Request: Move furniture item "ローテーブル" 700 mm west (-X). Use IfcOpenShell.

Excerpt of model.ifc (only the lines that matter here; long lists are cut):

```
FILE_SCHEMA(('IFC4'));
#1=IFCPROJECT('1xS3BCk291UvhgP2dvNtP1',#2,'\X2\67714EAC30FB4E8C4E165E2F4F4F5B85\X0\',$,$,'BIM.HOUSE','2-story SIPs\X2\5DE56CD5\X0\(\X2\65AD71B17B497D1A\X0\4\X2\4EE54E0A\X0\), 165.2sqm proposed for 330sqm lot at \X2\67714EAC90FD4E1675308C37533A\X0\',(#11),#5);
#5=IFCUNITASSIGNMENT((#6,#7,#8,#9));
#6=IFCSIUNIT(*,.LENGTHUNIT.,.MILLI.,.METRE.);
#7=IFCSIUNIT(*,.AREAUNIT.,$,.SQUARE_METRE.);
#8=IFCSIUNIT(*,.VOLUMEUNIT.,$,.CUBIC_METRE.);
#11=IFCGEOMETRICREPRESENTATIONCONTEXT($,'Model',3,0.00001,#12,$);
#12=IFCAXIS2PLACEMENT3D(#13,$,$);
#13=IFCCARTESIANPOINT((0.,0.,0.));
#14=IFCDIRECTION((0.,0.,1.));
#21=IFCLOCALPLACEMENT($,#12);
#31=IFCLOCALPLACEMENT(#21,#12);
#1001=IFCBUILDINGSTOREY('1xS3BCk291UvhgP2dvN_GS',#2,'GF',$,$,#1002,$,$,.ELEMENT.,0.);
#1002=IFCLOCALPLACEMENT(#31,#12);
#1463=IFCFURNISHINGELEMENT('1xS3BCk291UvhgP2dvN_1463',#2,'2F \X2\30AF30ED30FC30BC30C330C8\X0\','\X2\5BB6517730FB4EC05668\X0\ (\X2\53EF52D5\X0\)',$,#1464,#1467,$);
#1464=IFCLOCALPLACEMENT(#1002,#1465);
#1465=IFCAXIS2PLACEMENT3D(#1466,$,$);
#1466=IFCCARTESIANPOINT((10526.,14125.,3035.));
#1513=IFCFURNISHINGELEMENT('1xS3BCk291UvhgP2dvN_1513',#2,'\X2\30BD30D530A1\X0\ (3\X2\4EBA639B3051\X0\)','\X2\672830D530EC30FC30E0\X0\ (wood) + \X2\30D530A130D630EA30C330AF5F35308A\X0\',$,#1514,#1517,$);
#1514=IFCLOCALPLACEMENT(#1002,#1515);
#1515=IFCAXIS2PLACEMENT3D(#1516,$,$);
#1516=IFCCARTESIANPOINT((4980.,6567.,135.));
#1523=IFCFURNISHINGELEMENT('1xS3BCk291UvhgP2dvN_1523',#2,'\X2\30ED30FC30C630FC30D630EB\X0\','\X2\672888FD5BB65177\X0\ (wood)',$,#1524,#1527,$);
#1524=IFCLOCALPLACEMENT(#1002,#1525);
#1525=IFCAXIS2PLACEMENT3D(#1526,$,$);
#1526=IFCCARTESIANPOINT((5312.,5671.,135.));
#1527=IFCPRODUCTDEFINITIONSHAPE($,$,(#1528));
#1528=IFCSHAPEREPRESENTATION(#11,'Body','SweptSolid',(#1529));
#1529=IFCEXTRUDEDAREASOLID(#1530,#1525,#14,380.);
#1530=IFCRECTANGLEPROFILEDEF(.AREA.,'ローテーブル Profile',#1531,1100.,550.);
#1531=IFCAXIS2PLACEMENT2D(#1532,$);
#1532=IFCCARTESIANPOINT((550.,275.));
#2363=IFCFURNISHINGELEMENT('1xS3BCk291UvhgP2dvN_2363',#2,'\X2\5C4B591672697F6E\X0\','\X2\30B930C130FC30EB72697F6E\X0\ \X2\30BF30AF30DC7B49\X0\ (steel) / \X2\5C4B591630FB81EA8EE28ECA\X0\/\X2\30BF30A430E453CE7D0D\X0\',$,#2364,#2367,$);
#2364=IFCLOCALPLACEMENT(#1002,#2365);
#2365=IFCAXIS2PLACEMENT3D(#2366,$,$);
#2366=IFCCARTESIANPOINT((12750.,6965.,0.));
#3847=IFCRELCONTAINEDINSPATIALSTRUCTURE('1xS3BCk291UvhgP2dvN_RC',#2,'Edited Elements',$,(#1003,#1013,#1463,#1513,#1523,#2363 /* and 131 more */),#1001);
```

```python
import ifcopenshell
import ifcopenshell.api.geometry
import ifcopenshell.util.placement
import ifcopenshell.util.unit

model = ifcopenshell.open("model.ifc")
unit_scale = ifcopenshell.util.unit.calculate_unit_scale(model)

item = model.by_guid("1xS3BCk291UvhgP2dvN_1523")
matrix = ifcopenshell.util.placement.get_local_placement(item.ObjectPlacement)
matrix[0, 3] -= 0.7 / unit_scale
ifcopenshell.api.geometry.edit_object_placement(model, product=item, matrix=matrix, is_si=False)

print(ifcopenshell.util.placement.get_local_placement(item.ObjectPlacement).round(3) + 0.0)

model.write("model_v2.ifc")
```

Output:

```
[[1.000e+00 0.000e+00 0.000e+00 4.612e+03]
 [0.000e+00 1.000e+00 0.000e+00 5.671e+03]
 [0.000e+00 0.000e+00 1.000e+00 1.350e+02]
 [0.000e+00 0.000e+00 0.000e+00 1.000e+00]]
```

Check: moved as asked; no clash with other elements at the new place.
